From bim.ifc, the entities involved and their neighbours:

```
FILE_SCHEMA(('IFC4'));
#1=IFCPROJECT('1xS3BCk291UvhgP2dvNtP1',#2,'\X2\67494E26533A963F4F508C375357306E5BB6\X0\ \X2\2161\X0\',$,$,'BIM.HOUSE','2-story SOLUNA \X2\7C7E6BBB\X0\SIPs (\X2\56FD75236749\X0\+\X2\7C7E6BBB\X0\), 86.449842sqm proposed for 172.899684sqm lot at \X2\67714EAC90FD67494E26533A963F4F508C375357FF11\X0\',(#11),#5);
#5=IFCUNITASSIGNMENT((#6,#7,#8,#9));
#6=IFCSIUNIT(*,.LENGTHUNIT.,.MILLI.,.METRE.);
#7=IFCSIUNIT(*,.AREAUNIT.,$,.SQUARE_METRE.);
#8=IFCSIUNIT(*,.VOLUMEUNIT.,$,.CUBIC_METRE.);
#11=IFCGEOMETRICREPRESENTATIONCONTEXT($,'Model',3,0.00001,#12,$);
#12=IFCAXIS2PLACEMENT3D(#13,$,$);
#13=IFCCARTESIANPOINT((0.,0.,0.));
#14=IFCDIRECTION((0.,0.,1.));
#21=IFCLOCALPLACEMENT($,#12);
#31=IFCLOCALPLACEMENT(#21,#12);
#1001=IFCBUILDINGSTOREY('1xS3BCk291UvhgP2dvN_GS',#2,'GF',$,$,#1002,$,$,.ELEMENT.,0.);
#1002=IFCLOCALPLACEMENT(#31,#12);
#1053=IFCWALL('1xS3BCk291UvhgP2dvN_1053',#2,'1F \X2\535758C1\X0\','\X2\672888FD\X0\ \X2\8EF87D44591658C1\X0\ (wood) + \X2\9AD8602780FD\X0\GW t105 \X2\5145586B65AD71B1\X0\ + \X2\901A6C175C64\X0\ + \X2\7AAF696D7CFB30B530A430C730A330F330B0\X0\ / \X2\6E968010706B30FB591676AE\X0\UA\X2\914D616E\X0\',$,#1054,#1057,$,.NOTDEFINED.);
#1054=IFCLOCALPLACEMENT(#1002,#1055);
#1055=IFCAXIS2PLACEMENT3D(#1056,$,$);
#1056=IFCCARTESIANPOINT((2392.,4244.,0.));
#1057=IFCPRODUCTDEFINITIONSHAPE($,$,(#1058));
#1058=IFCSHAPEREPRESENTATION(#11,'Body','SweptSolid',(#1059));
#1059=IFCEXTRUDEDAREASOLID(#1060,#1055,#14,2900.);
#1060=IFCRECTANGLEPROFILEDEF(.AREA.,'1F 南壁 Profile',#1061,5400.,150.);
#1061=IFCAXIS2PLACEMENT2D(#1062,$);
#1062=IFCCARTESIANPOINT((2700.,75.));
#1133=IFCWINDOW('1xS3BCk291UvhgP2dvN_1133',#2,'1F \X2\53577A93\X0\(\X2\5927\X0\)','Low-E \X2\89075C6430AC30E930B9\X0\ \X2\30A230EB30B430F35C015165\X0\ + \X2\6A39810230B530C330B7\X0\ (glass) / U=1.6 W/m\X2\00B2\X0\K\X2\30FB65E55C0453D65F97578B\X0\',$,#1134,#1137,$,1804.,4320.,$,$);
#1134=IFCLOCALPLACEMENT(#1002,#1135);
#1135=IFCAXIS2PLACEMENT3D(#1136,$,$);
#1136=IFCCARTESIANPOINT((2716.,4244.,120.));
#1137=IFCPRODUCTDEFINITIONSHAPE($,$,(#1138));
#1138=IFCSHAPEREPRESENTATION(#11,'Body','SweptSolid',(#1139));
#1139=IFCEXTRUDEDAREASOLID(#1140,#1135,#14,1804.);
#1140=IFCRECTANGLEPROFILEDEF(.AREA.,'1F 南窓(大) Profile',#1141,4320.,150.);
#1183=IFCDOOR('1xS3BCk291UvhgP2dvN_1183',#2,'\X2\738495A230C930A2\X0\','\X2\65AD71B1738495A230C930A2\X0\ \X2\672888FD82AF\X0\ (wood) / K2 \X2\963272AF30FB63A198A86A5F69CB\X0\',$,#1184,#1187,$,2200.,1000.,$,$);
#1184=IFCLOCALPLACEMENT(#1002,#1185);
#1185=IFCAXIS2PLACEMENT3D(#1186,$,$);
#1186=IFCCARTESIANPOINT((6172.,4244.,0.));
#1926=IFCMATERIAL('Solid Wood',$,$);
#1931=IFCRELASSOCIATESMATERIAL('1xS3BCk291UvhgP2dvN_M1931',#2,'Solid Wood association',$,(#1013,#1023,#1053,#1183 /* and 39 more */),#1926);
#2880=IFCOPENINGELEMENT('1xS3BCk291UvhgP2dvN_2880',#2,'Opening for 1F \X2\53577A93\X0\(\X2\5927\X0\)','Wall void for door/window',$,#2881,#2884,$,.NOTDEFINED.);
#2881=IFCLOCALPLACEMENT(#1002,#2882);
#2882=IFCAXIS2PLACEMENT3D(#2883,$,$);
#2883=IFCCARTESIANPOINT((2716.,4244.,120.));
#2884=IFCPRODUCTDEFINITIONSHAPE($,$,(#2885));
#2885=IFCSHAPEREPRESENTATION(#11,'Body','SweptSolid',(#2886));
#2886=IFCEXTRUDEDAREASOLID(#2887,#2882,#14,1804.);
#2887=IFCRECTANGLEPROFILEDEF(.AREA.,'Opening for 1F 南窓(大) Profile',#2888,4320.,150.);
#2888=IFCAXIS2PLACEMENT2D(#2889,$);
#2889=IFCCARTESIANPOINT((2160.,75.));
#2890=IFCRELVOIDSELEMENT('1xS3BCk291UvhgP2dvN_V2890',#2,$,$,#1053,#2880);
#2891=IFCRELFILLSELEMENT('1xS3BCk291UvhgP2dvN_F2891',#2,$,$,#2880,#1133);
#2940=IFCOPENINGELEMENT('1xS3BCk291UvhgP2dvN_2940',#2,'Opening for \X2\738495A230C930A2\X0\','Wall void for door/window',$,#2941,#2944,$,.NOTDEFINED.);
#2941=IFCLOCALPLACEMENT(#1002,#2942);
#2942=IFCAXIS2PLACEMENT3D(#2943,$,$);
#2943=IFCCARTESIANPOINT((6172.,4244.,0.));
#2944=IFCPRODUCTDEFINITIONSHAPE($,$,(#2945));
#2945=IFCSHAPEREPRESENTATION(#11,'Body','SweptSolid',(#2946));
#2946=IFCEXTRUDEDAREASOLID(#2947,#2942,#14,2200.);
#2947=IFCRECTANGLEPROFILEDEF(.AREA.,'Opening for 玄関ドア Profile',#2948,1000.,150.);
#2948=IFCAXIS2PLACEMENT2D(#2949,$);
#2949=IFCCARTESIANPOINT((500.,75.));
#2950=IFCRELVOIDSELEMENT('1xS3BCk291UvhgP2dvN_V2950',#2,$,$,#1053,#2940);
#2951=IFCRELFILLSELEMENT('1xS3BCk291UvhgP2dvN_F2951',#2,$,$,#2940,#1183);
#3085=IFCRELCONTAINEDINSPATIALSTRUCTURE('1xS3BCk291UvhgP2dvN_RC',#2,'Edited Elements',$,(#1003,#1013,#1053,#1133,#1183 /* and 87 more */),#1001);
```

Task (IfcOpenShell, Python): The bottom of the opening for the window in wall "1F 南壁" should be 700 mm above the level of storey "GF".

```python
import numpy as np
import ifcopenshell
import ifcopenshell.api.geometry
import ifcopenshell.geom
import ifcopenshell.util.element
import ifcopenshell.util.placement
import ifcopenshell.util.shape
import ifcopenshell.util.unit

model = ifcopenshell.open("bim.ifc")
unit_scale = ifcopenshell.util.unit.calculate_unit_scale(model)

window = model.by_guid("1xS3BCk291UvhgP2dvN_1133")
opening = window.FillsVoids[0].RelatingOpeningElement
storey = ifcopenshell.util.element.get_container(window, ifc_class="IfcBuildingStorey")
level = ifcopenshell.util.placement.get_local_placement(storey.ObjectPlacement)[2, 3]

# The opening's origin need not be at the sill, so measure its lowest point.
shape = ifcopenshell.geom.create_shape(ifcopenshell.geom.settings(), opening)
bottom = ifcopenshell.util.shape.get_shape_bottom_elevation(shape, shape.geometry) / unit_scale
dz = level + 0.7 / unit_scale - bottom

shift = np.array([0.0, 0.0, dz])
# The window is not placed relative to its opening, so move both.
for product in (opening, window):
    matrix = ifcopenshell.util.placement.get_local_placement(product.ObjectPlacement)
    matrix[:3, 3] += shift
    ifcopenshell.api.geometry.edit_object_placement(model, product=product, matrix=matrix, is_si=False)

print(f"moved by {dz * unit_scale:+.3f} m")

model.write("bim-out.ifc")
```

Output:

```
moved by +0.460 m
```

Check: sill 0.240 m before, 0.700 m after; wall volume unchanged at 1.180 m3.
